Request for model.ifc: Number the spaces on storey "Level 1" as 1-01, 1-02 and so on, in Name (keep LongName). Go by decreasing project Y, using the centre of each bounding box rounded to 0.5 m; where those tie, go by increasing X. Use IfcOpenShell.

First a look at what the model holds.

```python
import ifcopenshell
import ifcopenshell.util.element
import ifcopenshell.util.placement

model = ifcopenshell.open("model.ifc")
print(model.schema)
storey = next(s for s in model.by_type("IfcBuildingStorey") if s.Name == "Level 1")
spaces = [e for e in ifcopenshell.util.element.get_decomposition(storey) if e.is_a("IfcSpace")]
for e in sorted(spaces, key=lambda e: e.id()):
    origin = ifcopenshell.util.placement.get_local_placement(e.ObjectPlacement)[:3, 3]
    print(e.id(), e.Name, e.LongName, origin.round(2) + 0.0, sep=" | ")
```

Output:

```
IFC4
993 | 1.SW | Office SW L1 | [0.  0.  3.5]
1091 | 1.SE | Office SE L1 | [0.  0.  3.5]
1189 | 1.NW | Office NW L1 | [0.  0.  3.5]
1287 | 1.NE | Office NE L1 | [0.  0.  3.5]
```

```python
import ifcopenshell
import ifcopenshell.geom
import ifcopenshell.util.element
import ifcopenshell.util.shape

model = ifcopenshell.open("model.ifc")
settings = ifcopenshell.geom.settings()
settings.set("use-world-coords", True)


def centre(element):
    shape = ifcopenshell.geom.create_shape(settings, element)
    return ifcopenshell.util.shape.get_bbox_centroid(shape.geometry)


storey = next(s for s in model.by_type("IfcBuildingStorey") if s.Name == "Level 1")
spaces = [e for e in ifcopenshell.util.element.get_decomposition(storey) if e.is_a("IfcSpace")]

# Insertion points can sit at a corner or the storey origin, so sort by the geometry (in metres).
centres = {e: centre(e) for e in spaces}
spaces.sort(key=lambda e: (-round(centres[e][1] / 0.5), centres[e][0]))

for i, e in enumerate(spaces, start=1):
    number = f"1-{i:02d}"
    e.Name = number
    print(e.id(), number)

model.write("model_v2.ifc")
```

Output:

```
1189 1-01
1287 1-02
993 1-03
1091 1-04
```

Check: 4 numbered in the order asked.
